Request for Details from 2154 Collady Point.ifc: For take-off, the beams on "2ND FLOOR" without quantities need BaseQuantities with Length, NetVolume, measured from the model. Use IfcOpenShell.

First a look at what the model holds.

```python
import ifcopenshell
import ifcopenshell.util.element
import ifcopenshell.util.unit

model = ifcopenshell.open("Details from 2154 Collady Point.ifc")
print(model.schema)
for unit_type in ("LENGTHUNIT", "AREAUNIT", "VOLUMEUNIT"):
    print(unit_type, ifcopenshell.util.unit.calculate_unit_scale(model, unit_type))
storey = next(s for s in model.by_type("IfcBuildingStorey") if s.Name == "2ND FLOOR")
beams = [e for e in ifcopenshell.util.element.get_decomposition(storey) if e.is_a("IfcBeam")]
for e in sorted(beams, key=lambda e: e.id()):
    print(e.id(), e.is_a(), e.Name, list(ifcopenshell.util.element.get_psets(e, qtos_only=True)), sep=" | ")
```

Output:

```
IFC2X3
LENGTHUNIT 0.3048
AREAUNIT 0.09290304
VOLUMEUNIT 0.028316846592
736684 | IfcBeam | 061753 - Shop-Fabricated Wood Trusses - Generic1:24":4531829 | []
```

```python
import ifcopenshell
import ifcopenshell.api.pset
import ifcopenshell.geom
import ifcopenshell.util.element
import ifcopenshell.util.shape
import ifcopenshell.util.unit

model = ifcopenshell.open("Details from 2154 Collady Point.ifc")
unit_scale = ifcopenshell.util.unit.calculate_unit_scale(model)
volume_scale = ifcopenshell.util.unit.calculate_unit_scale(model, "VOLUMEUNIT")
settings = ifcopenshell.geom.settings()

storey = next(s for s in model.by_type("IfcBuildingStorey") if s.Name == "2ND FLOOR")
beams = [e for e in ifcopenshell.util.element.get_decomposition(storey) if e.is_a("IfcBeam")]

for e in sorted(beams, key=lambda e: e.id()):
    if ifcopenshell.util.element.get_psets(e, qtos_only=True, should_inherit=False):
        continue
    # Geometry comes back in metres, in the element's own axes.
    shape = ifcopenshell.geom.create_shape(settings, e)
    values = {
        "Length": ifcopenshell.util.shape.get_max_xyz(shape.geometry) / unit_scale,
        "NetVolume": ifcopenshell.util.shape.get_volume(shape.geometry) / volume_scale,
    }
    qto = ifcopenshell.api.pset.add_qto(model, product=e, name="BaseQuantities")
    ifcopenshell.api.pset.edit_qto(model, qto=qto, properties=values)
    print(e.id(), {k: round(v, 3) for k, v in values.items()})

model.write("Details from 2154 Collady Point_v2.ifc")
```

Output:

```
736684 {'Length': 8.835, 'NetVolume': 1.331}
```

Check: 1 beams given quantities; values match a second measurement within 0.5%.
